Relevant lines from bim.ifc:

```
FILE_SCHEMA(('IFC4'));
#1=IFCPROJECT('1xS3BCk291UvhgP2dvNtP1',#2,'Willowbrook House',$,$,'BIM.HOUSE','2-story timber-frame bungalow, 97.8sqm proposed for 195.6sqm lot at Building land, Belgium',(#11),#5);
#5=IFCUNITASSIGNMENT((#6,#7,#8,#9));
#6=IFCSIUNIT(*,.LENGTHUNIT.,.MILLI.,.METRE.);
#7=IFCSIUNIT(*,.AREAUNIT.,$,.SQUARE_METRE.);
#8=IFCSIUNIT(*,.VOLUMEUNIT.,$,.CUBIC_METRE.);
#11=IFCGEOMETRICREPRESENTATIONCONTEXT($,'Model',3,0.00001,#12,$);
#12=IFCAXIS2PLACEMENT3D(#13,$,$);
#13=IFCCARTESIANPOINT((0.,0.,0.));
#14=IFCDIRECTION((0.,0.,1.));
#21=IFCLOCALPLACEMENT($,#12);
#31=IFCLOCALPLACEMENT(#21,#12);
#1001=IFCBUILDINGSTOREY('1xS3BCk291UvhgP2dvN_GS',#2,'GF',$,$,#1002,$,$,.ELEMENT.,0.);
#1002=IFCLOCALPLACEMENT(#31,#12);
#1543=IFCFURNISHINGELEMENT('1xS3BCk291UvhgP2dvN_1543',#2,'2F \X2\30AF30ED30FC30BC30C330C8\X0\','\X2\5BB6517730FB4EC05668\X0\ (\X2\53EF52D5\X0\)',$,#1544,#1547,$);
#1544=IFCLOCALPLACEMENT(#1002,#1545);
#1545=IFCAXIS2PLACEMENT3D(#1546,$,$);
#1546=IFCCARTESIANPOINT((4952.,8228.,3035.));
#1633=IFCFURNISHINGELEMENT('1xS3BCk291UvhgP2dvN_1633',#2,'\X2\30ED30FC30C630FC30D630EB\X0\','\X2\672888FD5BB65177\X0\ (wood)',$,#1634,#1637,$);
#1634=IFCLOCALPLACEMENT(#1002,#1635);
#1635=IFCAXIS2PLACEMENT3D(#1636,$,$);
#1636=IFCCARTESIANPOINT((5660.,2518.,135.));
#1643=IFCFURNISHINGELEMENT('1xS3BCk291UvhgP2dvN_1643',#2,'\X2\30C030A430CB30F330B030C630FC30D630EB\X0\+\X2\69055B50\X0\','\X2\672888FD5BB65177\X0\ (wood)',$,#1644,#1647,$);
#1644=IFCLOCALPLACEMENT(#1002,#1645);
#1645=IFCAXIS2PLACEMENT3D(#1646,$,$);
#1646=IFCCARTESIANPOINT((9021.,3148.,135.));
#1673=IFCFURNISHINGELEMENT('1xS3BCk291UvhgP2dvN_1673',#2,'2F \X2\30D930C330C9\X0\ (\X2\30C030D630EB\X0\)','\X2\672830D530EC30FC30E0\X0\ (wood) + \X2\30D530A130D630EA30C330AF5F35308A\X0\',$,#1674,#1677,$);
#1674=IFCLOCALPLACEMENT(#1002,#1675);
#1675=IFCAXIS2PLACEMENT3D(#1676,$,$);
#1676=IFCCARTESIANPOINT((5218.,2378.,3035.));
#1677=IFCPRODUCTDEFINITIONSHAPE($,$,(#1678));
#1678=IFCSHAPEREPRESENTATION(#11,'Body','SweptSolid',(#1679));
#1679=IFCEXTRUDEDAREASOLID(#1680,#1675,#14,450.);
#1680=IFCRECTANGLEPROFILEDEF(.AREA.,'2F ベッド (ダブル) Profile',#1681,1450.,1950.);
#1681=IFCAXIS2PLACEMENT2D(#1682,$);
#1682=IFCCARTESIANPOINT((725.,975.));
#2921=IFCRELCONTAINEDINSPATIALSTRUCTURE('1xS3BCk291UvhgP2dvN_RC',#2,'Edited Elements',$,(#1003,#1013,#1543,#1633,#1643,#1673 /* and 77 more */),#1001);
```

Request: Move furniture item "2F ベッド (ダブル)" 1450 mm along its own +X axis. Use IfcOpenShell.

```python
import ifcopenshell
import ifcopenshell.api.geometry
import ifcopenshell.util.placement
import ifcopenshell.util.unit

model = ifcopenshell.open("bim.ifc")
unit_scale = ifcopenshell.util.unit.calculate_unit_scale(model)

item = model.by_id(1673)
matrix = ifcopenshell.util.placement.get_local_placement(item.ObjectPlacement)
matrix[:3, 3] += matrix[:3, 0] * 1.45 / unit_scale
ifcopenshell.api.geometry.edit_object_placement(model, product=item, matrix=matrix, is_si=False)

print(ifcopenshell.util.placement.get_local_placement(item.ObjectPlacement).round(3) + 0.0)

model.write("bim_rev.ifc")
```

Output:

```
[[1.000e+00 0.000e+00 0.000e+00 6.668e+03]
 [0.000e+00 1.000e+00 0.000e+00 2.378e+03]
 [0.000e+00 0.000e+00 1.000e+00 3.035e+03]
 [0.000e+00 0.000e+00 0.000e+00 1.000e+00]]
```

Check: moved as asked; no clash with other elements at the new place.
